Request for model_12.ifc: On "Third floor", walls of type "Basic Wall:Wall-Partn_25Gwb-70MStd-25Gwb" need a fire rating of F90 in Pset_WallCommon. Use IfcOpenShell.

First a look at what the model holds.

```python
import ifcopenshell
import ifcopenshell.util.element

model = ifcopenshell.open("model_12.ifc")
print(model.schema)
storey = next(s for s in model.by_type("IfcBuildingStorey") if s.Name == "Third floor")
walls = [e for e in ifcopenshell.util.element.get_decomposition(storey) if e.is_a("IfcWall")]
seen = {}
for e in walls:
    element_type = ifcopenshell.util.element.get_type(e)
    key = (element_type.Name if element_type != e and element_type else None, ifcopenshell.util.element.get_pset(e, "Pset_WallCommon", "FireRating"))
    seen[key] = seen.get(key, 0) + 1
for (name, value), count in sorted(seen.items(), key=str):
    print(count, "x", name, "|", value)
```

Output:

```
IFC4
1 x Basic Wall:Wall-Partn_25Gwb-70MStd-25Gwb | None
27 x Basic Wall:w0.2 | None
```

```python
import ifcopenshell
import ifcopenshell.api.pset
import ifcopenshell.util.element

model = ifcopenshell.open("model_12.ifc")

storey = next(s for s in model.by_type("IfcBuildingStorey") if s.Name == "Third floor")
walls = [e for e in ifcopenshell.util.element.get_decomposition(storey) if e.is_a("IfcWall")]

count = 0
for e in walls:
    element_type = ifcopenshell.util.element.get_type(e)
    if element_type in (None, e) or element_type.Name != "Basic Wall:Wall-Partn_25Gwb-70MStd-25Gwb":
        continue
    # add_pset returns the element's existing set when there is one.
    pset = ifcopenshell.api.pset.add_pset(model, product=e, name="Pset_WallCommon")
    ifcopenshell.api.pset.edit_pset(model, pset=pset, properties={"FireRating": "F90"})
    count += 1

print(count, "walls updated")

model.write("model_12-out.ifc")
```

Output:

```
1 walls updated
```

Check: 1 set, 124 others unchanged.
